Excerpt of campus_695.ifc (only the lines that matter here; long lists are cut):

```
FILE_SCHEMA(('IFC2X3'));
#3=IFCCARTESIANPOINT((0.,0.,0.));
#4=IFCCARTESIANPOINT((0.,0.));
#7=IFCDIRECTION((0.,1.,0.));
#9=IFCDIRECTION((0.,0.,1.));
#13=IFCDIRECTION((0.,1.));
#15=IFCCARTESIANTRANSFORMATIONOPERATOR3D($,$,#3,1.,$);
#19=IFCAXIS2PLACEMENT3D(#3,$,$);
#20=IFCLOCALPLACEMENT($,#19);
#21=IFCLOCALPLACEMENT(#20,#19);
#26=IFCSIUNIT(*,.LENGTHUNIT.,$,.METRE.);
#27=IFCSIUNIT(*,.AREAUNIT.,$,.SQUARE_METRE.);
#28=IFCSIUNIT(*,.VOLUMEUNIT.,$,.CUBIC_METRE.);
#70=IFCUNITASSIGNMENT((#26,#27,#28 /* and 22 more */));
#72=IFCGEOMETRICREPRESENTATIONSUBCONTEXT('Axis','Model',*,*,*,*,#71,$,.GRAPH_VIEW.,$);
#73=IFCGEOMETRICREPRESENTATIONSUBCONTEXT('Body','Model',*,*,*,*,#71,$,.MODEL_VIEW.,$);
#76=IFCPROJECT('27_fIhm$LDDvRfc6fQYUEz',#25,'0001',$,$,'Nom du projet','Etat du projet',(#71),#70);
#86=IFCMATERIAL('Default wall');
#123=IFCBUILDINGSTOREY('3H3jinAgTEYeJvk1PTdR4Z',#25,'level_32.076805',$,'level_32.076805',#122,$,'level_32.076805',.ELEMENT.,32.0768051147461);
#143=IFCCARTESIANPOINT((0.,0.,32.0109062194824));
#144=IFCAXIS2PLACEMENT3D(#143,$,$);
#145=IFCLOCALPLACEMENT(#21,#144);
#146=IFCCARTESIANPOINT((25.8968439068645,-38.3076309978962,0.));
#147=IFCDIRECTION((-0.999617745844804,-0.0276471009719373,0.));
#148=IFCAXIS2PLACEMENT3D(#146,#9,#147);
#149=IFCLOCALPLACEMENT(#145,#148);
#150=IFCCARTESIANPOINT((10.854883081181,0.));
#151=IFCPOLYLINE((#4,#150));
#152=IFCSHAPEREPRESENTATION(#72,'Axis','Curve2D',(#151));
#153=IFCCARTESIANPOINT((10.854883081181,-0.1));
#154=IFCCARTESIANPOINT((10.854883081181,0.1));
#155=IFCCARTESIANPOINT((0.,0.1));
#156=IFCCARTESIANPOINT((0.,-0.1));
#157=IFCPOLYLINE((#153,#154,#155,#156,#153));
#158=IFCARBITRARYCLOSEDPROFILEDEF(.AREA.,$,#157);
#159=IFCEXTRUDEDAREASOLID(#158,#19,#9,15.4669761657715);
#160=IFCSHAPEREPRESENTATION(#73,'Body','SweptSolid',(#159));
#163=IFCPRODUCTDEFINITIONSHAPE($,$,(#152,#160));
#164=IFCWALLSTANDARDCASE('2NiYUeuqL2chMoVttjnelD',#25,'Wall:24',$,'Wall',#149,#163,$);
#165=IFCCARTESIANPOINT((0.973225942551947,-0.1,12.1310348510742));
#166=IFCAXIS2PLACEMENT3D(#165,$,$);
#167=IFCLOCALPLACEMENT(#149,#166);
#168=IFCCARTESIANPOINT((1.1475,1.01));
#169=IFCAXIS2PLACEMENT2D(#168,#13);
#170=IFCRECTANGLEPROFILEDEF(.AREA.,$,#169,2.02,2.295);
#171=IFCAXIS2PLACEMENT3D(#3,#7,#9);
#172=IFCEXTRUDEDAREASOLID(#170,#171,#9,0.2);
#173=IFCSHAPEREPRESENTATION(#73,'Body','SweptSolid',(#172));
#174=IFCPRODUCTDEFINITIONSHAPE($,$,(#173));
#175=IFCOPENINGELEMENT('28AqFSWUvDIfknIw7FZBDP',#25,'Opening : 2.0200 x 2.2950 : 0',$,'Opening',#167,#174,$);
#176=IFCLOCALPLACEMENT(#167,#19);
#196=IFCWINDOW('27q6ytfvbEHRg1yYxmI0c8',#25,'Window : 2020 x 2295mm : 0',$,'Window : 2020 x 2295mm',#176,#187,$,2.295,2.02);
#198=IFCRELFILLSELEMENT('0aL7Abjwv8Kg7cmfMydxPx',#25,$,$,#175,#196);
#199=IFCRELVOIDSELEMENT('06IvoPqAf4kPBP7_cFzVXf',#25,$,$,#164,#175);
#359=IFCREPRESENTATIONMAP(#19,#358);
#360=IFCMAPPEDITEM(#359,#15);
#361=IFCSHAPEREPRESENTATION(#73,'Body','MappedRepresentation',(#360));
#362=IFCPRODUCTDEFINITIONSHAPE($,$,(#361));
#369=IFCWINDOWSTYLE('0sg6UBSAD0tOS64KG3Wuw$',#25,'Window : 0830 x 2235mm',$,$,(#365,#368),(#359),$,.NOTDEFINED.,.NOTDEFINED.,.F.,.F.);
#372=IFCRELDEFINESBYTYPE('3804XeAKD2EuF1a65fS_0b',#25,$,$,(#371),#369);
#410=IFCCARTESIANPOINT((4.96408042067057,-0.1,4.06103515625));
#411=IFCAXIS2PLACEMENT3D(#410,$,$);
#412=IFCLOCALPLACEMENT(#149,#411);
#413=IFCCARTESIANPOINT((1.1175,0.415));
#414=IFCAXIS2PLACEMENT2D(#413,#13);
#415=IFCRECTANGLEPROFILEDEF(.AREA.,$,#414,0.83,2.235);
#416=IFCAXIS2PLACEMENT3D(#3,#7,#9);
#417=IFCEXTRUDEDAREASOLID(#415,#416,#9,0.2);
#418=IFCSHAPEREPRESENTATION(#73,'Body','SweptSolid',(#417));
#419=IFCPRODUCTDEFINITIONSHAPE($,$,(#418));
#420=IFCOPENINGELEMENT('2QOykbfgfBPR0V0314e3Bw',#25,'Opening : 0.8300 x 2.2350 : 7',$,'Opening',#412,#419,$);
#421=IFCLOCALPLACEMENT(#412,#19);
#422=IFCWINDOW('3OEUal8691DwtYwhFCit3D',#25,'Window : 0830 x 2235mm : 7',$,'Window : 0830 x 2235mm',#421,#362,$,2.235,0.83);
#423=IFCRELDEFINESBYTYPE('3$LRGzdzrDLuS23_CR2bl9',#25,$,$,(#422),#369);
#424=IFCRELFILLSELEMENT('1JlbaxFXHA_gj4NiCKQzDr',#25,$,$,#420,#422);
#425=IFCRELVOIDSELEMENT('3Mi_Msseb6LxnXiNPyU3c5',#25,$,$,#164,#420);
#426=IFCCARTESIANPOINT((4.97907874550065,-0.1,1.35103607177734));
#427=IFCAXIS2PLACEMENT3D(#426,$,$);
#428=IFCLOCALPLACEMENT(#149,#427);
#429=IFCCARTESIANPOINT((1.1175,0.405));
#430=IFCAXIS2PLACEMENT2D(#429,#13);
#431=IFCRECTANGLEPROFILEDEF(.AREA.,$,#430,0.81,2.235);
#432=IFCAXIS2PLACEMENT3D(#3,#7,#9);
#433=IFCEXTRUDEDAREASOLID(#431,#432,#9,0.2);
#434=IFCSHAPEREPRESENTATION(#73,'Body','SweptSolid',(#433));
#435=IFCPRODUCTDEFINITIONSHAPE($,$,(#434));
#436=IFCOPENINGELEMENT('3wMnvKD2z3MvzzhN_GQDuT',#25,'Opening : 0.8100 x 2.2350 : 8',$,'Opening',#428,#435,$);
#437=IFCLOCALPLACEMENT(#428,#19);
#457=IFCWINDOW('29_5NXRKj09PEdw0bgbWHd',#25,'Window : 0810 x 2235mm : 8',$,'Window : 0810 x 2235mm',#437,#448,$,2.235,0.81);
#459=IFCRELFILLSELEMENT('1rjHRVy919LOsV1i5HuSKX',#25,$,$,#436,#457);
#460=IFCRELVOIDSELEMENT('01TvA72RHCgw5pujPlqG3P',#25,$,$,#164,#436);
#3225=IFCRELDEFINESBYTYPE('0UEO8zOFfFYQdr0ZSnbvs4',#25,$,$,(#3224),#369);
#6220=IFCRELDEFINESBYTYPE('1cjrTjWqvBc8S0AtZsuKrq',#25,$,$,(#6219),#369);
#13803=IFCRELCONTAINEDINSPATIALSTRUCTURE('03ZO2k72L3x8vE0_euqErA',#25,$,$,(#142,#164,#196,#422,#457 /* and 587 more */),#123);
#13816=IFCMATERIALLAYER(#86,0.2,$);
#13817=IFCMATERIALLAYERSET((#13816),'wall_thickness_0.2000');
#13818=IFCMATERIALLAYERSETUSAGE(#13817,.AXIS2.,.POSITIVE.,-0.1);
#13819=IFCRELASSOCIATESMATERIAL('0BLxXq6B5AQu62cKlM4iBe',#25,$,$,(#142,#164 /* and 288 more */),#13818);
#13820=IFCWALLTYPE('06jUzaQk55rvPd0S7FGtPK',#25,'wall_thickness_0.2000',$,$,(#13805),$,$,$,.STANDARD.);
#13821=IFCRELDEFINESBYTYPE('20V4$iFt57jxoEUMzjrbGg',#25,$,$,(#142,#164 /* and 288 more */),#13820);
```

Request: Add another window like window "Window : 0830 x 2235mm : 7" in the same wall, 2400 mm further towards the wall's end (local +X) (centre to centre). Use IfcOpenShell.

```python
import ifcopenshell
import ifcopenshell.api.feature
import ifcopenshell.api.geometry
import ifcopenshell.api.root
import ifcopenshell.geom
import ifcopenshell.util.element
import ifcopenshell.util.placement
import ifcopenshell.util.shape
import ifcopenshell.util.unit

model = ifcopenshell.open("campus_695.ifc")
unit_scale = ifcopenshell.util.unit.calculate_unit_scale(model)
settings = ifcopenshell.geom.settings()


def volume(element):
    """Net volume in cubic metres, openings subtracted."""
    shape = ifcopenshell.geom.create_shape(settings, element)
    return ifcopenshell.util.shape.get_volume(shape.geometry)


window = model.by_guid("3OEUal8691DwtYwhFCit3D")
opening = window.FillsVoids[0].RelatingOpeningElement
wall = opening.VoidsElements[0].RelatingBuildingElement
before = volume(wall)
shift = ifcopenshell.util.placement.get_local_placement(wall.ObjectPlacement)[:3, 0] * 2.4 / unit_scale

# copy_class copies the void relationship, type, container and properties, but no geometry.
new_opening = ifcopenshell.api.root.copy_class(model, product=opening)
new_opening.Representation = ifcopenshell.util.element.copy_deep(
    model, opening.Representation, exclude=["IfcGeometricRepresentationContext", "IfcRepresentationMap"]
)
new_opening.Name = "Opening : 0.8300 x 2.2350"
new_window = ifcopenshell.api.root.copy_class(model, product=window)
new_window.Representation = ifcopenshell.util.element.copy_deep(
    model, window.Representation, exclude=["IfcGeometricRepresentationContext", "IfcRepresentationMap"]
)
new_window.Name = "Window : 0830 x 2235mm"
fills = ifcopenshell.api.feature.add_filling(model, opening=new_opening, element=new_window)
fills.OwnerHistory = new_window.OwnerHistory  # required in IFC2X3

for old, new in ((opening, new_opening), (window, new_window)):
    matrix = ifcopenshell.util.placement.get_local_placement(old.ObjectPlacement)
    matrix[:3, 3] += shift
    ifcopenshell.api.geometry.edit_object_placement(model, product=new, matrix=matrix, is_si=False)

after = volume(wall)

print(f"wall volume {before:.3f} -> {after:.3f} m3")

model.write("campus_695_rev.ifc")
```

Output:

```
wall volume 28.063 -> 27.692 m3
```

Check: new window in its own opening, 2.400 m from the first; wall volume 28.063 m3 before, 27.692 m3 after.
